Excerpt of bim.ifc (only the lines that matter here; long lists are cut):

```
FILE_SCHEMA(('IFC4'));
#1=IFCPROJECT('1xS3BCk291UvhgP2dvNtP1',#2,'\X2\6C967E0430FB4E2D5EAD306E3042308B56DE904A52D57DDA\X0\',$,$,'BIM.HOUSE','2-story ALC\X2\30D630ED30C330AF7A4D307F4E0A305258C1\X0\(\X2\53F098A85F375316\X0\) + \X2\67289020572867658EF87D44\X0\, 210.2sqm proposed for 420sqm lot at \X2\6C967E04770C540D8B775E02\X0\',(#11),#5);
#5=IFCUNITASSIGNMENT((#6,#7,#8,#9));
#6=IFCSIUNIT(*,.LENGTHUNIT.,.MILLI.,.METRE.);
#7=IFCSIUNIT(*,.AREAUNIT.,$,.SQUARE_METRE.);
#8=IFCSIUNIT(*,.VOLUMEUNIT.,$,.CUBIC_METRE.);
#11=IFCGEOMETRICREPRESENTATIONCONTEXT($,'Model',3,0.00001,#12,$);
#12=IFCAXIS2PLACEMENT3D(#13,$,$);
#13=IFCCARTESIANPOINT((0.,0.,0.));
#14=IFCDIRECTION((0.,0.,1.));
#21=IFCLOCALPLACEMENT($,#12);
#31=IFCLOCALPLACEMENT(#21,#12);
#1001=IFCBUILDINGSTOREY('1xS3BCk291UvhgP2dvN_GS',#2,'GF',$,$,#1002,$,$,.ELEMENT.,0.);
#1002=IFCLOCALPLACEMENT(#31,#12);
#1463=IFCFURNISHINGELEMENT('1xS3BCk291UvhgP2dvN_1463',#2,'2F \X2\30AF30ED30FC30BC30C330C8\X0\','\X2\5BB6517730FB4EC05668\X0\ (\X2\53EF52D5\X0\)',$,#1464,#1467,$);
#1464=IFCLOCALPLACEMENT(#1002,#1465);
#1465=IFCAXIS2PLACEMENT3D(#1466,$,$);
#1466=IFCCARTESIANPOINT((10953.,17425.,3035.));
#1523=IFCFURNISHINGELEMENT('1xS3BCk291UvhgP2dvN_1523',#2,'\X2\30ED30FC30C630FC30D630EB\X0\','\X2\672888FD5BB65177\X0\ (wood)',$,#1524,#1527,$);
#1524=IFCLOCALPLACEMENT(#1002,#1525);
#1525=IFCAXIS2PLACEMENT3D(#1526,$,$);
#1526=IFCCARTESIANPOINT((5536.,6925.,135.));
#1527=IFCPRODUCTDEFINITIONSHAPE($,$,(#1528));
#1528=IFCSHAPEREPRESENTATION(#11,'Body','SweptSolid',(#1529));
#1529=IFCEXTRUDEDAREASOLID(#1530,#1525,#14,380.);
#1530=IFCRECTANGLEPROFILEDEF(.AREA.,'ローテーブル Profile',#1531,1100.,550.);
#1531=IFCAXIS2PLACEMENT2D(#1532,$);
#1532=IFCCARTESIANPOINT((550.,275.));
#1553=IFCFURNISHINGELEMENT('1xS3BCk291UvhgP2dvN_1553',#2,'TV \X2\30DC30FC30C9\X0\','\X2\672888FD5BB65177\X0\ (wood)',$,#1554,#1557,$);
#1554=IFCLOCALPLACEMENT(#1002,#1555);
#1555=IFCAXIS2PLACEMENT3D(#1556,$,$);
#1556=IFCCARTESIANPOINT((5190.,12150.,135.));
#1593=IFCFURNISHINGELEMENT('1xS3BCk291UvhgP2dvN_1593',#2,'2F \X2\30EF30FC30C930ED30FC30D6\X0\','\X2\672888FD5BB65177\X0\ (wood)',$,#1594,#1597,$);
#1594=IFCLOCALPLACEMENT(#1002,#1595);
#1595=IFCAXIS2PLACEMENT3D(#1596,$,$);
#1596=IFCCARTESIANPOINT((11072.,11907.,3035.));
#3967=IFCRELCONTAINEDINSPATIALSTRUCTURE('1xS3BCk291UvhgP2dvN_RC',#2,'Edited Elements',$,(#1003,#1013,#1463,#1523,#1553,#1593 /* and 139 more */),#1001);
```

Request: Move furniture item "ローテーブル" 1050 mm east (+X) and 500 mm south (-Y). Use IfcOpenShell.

```python
import ifcopenshell
import ifcopenshell.api.geometry
import ifcopenshell.util.placement
import ifcopenshell.util.unit

model = ifcopenshell.open("bim.ifc")
unit_scale = ifcopenshell.util.unit.calculate_unit_scale(model)

item = model.by_id(1523)
matrix = ifcopenshell.util.placement.get_local_placement(item.ObjectPlacement)
matrix[0, 3] += 1.05 / unit_scale
matrix[1, 3] -= 0.5 / unit_scale
ifcopenshell.api.geometry.edit_object_placement(model, product=item, matrix=matrix, is_si=False)

print(ifcopenshell.util.placement.get_local_placement(item.ObjectPlacement).round(3) + 0.0)

model.write("bim_rev.ifc")
```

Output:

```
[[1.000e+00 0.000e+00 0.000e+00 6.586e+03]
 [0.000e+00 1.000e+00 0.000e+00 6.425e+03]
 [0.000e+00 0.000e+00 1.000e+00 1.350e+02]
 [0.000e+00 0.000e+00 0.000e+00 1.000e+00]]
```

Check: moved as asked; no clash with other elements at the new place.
